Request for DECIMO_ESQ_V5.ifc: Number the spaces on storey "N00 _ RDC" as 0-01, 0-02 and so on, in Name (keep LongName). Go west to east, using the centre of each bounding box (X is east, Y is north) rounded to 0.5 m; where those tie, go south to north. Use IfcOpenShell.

First a look at what the model holds.

```python
import ifcopenshell
import ifcopenshell.util.element
import ifcopenshell.util.placement

model = ifcopenshell.open("DECIMO_ESQ_V5.ifc")
print(model.schema)
storey = next(s for s in model.by_type("IfcBuildingStorey") if s.Name == "N00 _ RDC")
spaces = [e for e in ifcopenshell.util.element.get_decomposition(storey) if e.is_a("IfcSpace")]
for e in sorted(spaces, key=lambda e: e.id()):
    origin = ifcopenshell.util.placement.get_local_placement(e.ObjectPlacement)[:3, 3]
    print(e.id(), e.Name, e.LongName, origin.round(2) + 0.0, sep=" | ")
```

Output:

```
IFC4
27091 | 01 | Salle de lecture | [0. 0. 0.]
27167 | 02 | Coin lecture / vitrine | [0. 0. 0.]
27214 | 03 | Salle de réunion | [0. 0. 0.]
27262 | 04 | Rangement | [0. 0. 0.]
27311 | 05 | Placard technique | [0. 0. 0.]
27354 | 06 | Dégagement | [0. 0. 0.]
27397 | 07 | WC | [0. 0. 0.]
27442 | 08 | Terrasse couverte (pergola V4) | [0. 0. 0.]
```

```python
import ifcopenshell
import ifcopenshell.geom
import ifcopenshell.util.element
import ifcopenshell.util.shape

model = ifcopenshell.open("DECIMO_ESQ_V5.ifc")
settings = ifcopenshell.geom.settings()
settings.set("use-world-coords", True)


def centre(element):
    shape = ifcopenshell.geom.create_shape(settings, element)
    return ifcopenshell.util.shape.get_bbox_centroid(shape.geometry)


storey = next(s for s in model.by_type("IfcBuildingStorey") if s.Name == "N00 _ RDC")
spaces = [e for e in ifcopenshell.util.element.get_decomposition(storey) if e.is_a("IfcSpace")]

# Insertion points can sit at a corner or the storey origin, so sort by the geometry (in metres).
centres = {e: centre(e) for e in spaces}
spaces.sort(key=lambda e: (round(centres[e][0] / 0.5), centres[e][1]))

for i, e in enumerate(spaces, start=1):
    number = f"0-{i:02d}"
    e.Name = number
    print(e.id(), number)

model.write("DECIMO_ESQ_V5_rev.ifc")
```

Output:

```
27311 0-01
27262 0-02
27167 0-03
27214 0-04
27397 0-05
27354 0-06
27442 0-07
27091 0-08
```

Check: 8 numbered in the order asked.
